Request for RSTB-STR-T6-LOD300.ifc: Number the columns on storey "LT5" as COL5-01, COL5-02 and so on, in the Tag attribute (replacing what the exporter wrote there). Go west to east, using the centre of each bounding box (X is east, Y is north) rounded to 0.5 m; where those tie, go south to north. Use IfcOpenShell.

First a look at what the model holds.

```python
import ifcopenshell
import ifcopenshell.util.element
import ifcopenshell.util.placement

model = ifcopenshell.open("RSTB-STR-T6-LOD300.ifc")
print(model.schema)
storey = next(s for s in model.by_type("IfcBuildingStorey") if s.Name == "LT5")
columns = [e for e in ifcopenshell.util.element.get_decomposition(storey) if e.is_a("IfcColumn")]
for e in sorted(columns, key=lambda e: e.id()):
    origin = ifcopenshell.util.placement.get_local_placement(e.ObjectPlacement)[:3, 3]
    print(e.id(), e.Tag, e.Name, origin.round(2) + 0.0, sep=" | ")
```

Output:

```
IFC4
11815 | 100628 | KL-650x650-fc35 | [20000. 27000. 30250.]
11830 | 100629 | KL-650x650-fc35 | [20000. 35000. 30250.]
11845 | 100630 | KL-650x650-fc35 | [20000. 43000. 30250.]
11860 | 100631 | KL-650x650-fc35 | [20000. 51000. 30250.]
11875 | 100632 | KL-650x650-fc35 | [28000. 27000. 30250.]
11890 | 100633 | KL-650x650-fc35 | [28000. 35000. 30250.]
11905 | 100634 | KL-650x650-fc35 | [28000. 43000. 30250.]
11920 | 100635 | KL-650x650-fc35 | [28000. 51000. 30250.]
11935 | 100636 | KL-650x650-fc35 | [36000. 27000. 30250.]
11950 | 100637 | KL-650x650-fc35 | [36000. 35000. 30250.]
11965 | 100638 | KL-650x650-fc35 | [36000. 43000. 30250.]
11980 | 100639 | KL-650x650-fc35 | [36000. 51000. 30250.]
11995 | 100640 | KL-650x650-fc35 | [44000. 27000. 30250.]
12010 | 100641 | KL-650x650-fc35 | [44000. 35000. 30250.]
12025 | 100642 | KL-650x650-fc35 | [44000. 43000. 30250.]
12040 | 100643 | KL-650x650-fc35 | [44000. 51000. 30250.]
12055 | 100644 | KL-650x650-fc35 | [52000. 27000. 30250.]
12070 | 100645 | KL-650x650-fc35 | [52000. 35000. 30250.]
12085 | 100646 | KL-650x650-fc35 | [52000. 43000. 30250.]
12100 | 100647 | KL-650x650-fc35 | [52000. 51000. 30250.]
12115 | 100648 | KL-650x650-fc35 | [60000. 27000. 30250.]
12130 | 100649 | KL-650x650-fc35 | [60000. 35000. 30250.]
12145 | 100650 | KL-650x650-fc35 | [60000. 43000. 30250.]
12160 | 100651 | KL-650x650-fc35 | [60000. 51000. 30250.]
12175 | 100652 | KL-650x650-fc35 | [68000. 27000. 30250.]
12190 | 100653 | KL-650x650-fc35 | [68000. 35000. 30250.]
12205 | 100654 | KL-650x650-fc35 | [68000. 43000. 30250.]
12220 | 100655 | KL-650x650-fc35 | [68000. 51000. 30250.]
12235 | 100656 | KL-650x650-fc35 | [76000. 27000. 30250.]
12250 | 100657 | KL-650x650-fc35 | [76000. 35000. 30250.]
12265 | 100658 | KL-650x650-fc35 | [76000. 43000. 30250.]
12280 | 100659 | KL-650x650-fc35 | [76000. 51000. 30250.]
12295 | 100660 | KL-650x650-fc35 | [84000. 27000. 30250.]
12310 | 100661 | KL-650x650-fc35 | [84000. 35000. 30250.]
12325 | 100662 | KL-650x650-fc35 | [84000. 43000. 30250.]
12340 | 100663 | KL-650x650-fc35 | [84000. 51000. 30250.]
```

```python
import ifcopenshell
import ifcopenshell.geom
import ifcopenshell.util.element
import ifcopenshell.util.shape

model = ifcopenshell.open("RSTB-STR-T6-LOD300.ifc")
settings = ifcopenshell.geom.settings()
settings.set("use-world-coords", True)


def centre(element):
    shape = ifcopenshell.geom.create_shape(settings, element)
    return ifcopenshell.util.shape.get_bbox_centroid(shape.geometry)


storey = next(s for s in model.by_type("IfcBuildingStorey") if s.Name == "LT5")
columns = [e for e in ifcopenshell.util.element.get_decomposition(storey) if e.is_a("IfcColumn")]

# Insertion points can sit at a corner or the storey origin, so sort by the geometry (in metres).
centres = {e: centre(e) for e in columns}
columns.sort(key=lambda e: (round(centres[e][0] / 0.5), centres[e][1]))

for i, e in enumerate(columns, start=1):
    number = f"COL5-{i:02d}"
    e.Tag = number
    print(e.id(), number)

model.write("RSTB-STR-T6-LOD300_edited.ifc")
```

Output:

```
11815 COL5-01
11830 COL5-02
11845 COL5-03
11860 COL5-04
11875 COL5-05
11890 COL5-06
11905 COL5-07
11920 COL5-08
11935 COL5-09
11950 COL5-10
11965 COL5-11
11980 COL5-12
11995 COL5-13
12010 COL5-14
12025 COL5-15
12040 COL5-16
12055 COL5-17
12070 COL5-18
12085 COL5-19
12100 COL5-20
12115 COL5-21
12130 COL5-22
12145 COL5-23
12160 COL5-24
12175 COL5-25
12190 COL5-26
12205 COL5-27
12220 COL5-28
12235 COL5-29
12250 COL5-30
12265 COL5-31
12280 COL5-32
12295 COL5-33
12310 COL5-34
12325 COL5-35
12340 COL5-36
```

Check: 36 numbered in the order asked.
